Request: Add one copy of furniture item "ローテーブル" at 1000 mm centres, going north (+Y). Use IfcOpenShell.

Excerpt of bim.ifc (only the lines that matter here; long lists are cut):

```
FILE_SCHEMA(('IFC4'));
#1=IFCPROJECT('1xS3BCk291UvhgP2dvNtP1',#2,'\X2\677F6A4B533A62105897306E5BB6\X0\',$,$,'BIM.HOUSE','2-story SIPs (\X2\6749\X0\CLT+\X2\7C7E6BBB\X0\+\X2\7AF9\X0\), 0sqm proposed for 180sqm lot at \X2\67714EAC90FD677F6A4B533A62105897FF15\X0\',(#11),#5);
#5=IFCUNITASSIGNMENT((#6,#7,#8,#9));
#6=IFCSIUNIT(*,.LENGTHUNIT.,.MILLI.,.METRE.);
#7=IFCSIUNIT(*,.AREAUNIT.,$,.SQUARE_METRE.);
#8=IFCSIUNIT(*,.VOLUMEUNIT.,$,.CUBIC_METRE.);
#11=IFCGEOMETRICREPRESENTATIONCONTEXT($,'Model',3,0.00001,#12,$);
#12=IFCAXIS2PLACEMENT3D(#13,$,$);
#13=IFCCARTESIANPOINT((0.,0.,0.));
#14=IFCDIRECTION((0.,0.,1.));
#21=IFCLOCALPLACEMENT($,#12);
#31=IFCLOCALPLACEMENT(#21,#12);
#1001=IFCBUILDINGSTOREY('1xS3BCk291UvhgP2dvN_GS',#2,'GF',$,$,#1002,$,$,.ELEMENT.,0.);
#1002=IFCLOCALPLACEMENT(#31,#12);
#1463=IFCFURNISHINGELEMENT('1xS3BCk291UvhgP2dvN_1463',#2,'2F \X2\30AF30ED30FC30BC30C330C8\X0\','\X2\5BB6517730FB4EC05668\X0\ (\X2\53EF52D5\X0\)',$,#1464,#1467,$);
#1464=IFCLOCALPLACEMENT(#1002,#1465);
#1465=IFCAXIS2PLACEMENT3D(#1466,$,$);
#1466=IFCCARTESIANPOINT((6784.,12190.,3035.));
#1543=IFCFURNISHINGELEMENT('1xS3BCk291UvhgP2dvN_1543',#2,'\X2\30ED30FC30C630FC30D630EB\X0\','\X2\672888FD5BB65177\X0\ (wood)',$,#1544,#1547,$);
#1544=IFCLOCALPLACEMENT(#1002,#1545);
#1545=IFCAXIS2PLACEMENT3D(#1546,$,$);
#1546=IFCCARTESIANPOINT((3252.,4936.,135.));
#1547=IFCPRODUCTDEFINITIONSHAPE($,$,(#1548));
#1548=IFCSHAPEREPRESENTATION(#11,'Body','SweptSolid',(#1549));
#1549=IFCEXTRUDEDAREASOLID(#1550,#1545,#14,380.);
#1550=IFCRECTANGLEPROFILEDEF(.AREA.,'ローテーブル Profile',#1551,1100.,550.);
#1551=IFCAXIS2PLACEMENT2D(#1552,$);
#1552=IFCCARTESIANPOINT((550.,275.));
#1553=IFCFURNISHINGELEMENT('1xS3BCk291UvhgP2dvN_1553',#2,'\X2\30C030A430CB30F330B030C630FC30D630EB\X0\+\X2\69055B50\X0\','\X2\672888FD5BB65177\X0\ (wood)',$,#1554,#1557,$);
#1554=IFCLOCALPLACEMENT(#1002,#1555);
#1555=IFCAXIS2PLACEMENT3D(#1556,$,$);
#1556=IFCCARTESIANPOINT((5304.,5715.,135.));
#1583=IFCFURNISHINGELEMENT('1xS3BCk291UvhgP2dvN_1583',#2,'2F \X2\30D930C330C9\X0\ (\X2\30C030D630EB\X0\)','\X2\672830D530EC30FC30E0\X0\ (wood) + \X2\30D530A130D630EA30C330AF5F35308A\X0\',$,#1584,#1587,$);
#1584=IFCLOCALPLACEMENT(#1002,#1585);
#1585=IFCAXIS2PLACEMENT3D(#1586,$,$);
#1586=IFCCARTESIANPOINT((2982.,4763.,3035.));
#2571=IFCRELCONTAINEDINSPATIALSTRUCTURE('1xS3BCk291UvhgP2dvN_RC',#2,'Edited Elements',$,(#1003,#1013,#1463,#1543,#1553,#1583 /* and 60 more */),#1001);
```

```python
import numpy as np
import ifcopenshell
import ifcopenshell.api.geometry
import ifcopenshell.api.root
import ifcopenshell.util.element
import ifcopenshell.util.placement
import ifcopenshell.util.unit

model = ifcopenshell.open("bim.ifc")
unit_scale = ifcopenshell.util.unit.calculate_unit_scale(model)


def reuse_history(source, copy):
    """copy_class also copies each property set's owner history, people and application; keep the originals."""
    for rel in copy.IsDefinedBy:
        if rel.is_a("IfcRelDefinesByProperties") and (history := rel.RelatingPropertyDefinition.OwnerHistory):
            rel.RelatingPropertyDefinition.OwnerHistory = source.OwnerHistory
            ifcopenshell.util.element.remove_deep2(model, history)


source = model.by_id(1543)
base = ifcopenshell.util.placement.get_local_placement(source.ObjectPlacement)
step = np.array([0.0, 1.0, 0.0]) * 1 / unit_scale

for i in range(1, 2):
    copy = ifcopenshell.api.root.copy_class(model, product=source)
    copy.Representation = ifcopenshell.util.element.copy_deep(
        model, source.Representation, exclude=["IfcGeometricRepresentationContext", "IfcRepresentationMap"]
    )
    reuse_history(source, copy)
    matrix = base.copy()
    matrix[:3, 3] += i * step
    print("added at", matrix[:3, 3].round(3) + 0.0)
    ifcopenshell.api.geometry.edit_object_placement(model, product=copy, matrix=matrix, is_si=False)

model.write("bim_rev.ifc")
```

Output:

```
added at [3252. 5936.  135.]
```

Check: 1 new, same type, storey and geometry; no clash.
